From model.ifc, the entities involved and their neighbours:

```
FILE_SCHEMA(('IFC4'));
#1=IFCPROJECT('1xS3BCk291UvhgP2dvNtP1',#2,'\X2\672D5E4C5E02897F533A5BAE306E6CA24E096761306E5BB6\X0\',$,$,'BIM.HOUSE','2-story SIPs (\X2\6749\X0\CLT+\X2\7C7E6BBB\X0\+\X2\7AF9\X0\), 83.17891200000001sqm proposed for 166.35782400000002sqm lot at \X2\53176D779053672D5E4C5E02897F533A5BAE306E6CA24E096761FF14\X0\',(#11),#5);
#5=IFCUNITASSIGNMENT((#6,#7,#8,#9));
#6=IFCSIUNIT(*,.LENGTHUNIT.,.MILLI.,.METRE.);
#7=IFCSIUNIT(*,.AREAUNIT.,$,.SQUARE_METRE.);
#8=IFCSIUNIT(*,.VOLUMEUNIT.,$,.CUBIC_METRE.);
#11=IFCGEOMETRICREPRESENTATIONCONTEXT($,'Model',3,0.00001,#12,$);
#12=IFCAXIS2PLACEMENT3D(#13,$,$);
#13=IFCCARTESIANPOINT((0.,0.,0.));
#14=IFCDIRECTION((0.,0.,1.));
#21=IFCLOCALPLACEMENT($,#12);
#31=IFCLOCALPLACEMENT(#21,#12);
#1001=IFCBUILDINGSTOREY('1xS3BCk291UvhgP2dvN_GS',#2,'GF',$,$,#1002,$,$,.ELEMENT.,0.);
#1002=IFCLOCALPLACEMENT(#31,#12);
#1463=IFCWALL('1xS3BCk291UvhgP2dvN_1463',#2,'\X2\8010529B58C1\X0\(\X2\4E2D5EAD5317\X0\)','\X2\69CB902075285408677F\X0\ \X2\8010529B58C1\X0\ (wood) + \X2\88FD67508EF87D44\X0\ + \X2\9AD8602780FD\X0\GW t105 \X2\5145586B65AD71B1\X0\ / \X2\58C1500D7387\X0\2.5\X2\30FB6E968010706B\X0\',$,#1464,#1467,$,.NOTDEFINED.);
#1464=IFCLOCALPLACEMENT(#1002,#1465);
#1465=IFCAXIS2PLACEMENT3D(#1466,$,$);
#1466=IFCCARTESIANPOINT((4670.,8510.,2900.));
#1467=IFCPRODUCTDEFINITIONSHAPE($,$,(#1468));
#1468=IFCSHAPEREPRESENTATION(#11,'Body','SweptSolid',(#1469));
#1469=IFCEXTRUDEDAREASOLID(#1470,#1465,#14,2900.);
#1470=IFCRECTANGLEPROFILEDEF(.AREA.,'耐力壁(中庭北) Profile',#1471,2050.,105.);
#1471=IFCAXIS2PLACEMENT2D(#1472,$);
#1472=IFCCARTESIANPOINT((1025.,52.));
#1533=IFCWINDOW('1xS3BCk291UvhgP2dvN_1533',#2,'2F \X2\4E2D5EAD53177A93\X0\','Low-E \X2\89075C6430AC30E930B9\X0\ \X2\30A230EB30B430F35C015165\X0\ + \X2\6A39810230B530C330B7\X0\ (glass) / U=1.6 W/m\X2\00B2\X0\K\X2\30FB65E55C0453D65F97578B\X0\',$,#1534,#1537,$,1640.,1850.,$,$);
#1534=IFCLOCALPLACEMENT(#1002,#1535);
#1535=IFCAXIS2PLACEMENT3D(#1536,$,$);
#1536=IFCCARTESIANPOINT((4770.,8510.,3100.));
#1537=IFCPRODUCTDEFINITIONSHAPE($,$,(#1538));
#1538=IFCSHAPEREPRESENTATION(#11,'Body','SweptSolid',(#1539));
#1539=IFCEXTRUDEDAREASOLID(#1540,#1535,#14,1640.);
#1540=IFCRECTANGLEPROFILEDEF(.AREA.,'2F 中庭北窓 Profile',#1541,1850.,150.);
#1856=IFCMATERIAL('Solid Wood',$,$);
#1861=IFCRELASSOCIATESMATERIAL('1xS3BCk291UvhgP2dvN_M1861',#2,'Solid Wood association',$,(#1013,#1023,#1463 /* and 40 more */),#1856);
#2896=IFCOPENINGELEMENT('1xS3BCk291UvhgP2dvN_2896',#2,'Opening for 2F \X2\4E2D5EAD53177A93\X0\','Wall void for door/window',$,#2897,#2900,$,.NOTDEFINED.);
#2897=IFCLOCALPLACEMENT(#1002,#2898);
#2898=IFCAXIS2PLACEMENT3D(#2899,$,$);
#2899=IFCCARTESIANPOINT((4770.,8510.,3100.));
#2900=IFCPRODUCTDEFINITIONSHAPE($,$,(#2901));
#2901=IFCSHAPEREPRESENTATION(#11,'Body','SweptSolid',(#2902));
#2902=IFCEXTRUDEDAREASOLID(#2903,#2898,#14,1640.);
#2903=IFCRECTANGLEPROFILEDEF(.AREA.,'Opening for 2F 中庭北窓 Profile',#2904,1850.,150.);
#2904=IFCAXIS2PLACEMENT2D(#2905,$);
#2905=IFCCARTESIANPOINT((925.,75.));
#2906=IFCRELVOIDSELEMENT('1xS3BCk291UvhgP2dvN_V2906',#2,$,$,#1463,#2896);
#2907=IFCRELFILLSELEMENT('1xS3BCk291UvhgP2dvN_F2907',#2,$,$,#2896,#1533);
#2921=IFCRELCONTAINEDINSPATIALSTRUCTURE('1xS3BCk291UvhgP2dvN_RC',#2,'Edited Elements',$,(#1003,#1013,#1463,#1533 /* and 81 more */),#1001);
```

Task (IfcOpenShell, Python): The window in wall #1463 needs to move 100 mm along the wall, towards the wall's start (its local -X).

```python
import ifcopenshell
import ifcopenshell.api.geometry
import ifcopenshell.util.placement

model = ifcopenshell.open("model.ifc")

window = model.by_id(1533)
opening = window.FillsVoids[0].RelatingOpeningElement
wall = opening.VoidsElements[0].RelatingBuildingElement

wall_matrix = ifcopenshell.util.placement.get_local_placement(wall.ObjectPlacement)
shift = wall_matrix[:3, 0] * -100.0
before = ifcopenshell.util.placement.get_local_placement(window.ObjectPlacement)[:3, 3].copy()

# The window is not placed relative to its opening, so move both.
for product in (opening, window):
    matrix = ifcopenshell.util.placement.get_local_placement(product.ObjectPlacement)
    matrix[:3, 3] += shift
    ifcopenshell.api.geometry.edit_object_placement(model, product=product, matrix=matrix, is_si=False)

after = ifcopenshell.util.placement.get_local_placement(window.ObjectPlacement)[:3, 3]
print("window moved by", (after - before).round(3) + 0.0)

model.write("model-out.ifc")
```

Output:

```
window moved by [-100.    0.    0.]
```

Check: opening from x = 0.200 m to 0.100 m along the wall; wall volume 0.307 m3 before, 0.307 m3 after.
